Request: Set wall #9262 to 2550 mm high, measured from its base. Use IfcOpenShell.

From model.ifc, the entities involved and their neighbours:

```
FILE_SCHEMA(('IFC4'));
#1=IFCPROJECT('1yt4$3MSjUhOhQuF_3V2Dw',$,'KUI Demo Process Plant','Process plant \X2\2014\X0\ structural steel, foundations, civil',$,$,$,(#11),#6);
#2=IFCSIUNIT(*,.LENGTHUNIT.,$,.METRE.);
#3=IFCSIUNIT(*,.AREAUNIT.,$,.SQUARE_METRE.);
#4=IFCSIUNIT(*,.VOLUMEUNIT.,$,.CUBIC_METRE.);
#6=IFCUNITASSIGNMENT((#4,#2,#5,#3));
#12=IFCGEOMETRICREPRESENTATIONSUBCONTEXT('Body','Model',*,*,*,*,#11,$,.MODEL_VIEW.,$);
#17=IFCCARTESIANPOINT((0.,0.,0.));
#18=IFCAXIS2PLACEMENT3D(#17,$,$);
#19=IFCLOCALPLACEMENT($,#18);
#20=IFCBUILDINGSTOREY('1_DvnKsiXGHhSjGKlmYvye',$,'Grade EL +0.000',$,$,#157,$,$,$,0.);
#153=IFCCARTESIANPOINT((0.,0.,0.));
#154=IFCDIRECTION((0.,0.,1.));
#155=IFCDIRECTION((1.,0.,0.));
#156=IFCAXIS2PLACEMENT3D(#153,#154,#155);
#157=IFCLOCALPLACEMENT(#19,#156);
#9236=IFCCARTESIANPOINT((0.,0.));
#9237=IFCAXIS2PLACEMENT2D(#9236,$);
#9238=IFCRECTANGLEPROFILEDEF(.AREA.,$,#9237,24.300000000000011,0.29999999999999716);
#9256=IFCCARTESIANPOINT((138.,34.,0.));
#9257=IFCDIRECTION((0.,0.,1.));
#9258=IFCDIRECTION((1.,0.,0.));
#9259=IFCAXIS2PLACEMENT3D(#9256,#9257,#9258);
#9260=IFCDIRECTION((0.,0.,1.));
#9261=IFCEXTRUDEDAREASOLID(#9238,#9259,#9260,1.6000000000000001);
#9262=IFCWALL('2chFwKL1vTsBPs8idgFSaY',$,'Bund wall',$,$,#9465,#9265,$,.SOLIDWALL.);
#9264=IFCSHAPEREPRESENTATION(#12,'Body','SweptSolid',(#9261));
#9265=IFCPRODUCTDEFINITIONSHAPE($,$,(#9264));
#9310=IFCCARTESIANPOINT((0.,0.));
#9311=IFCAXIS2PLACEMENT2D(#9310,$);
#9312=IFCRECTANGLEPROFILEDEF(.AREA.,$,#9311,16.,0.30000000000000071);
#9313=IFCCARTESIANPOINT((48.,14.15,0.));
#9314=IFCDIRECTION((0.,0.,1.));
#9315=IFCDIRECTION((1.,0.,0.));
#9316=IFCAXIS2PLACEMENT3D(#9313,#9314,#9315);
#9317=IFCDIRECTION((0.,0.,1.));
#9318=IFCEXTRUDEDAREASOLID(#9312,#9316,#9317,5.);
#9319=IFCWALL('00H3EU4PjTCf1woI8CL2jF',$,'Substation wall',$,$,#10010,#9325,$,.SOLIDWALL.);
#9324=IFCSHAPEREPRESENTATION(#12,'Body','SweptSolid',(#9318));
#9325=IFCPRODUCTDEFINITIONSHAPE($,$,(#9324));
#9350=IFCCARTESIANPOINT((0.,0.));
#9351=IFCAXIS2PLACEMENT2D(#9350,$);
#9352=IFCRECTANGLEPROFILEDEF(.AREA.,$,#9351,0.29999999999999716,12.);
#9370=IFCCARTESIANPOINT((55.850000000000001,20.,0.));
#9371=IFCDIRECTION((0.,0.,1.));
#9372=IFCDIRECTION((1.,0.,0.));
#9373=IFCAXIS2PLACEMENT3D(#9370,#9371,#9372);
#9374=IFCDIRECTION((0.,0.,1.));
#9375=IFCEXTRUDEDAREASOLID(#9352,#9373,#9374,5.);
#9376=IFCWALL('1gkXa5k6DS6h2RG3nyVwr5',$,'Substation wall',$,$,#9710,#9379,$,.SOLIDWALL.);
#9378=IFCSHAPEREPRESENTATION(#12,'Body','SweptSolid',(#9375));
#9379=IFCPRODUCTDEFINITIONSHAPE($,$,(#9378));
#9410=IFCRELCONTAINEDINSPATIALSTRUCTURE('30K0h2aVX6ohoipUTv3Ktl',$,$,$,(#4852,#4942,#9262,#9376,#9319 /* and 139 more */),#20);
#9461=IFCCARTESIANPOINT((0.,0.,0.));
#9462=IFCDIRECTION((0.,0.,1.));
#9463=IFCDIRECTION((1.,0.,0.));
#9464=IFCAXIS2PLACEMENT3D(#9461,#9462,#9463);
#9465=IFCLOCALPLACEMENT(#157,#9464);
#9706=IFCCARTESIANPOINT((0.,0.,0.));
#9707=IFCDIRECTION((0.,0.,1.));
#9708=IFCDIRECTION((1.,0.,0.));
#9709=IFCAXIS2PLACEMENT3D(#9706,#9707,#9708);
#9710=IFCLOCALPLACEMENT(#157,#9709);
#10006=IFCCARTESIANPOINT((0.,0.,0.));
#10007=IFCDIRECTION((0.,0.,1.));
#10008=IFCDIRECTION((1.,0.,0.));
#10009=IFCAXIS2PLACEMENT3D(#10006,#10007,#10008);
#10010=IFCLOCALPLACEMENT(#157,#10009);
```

```python
import ifcopenshell
import ifcopenshell.geom
import ifcopenshell.util.representation
import ifcopenshell.util.shape
import ifcopenshell.util.unit

model = ifcopenshell.open("model.ifc")
unit_scale = ifcopenshell.util.unit.calculate_unit_scale(model)
settings = ifcopenshell.geom.settings()


def volume(element):
    """Net volume in cubic metres, openings subtracted."""
    shape = ifcopenshell.geom.create_shape(settings, element)
    return ifcopenshell.util.shape.get_volume(shape.geometry)


wall = model.by_id(9262)
before = volume(wall)

body = ifcopenshell.util.representation.get_representation(wall, "Model", "Body")
solid = body.Items[0]
old_height = solid.Depth
solid.Depth = 2.55 / unit_scale
after = volume(wall)

print(f"height {old_height:g} -> {solid.Depth:g}, volume {before:.3f} -> {after:.3f} m3")

model.write("model_rev.ifc")
```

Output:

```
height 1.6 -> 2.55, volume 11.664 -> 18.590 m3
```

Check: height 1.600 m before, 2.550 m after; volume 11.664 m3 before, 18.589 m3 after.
